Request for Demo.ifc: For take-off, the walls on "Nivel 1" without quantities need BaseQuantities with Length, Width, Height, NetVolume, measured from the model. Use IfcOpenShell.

First a look at what the model holds.

```python
import ifcopenshell
import ifcopenshell.util.element
import ifcopenshell.util.unit

model = ifcopenshell.open("Demo.ifc")
print(model.schema)
for unit_type in ("LENGTHUNIT", "AREAUNIT", "VOLUMEUNIT"):
    print(unit_type, ifcopenshell.util.unit.calculate_unit_scale(model, unit_type))
storey = next(s for s in model.by_type("IfcBuildingStorey") if s.Name == "Nivel 1")
walls = [e for e in ifcopenshell.util.element.get_decomposition(storey) if e.is_a("IfcWall")]
for e in sorted(walls, key=lambda e: e.id()):
    print(e.id(), e.is_a(), e.Name, list(ifcopenshell.util.element.get_psets(e, qtos_only=True)), sep=" | ")
```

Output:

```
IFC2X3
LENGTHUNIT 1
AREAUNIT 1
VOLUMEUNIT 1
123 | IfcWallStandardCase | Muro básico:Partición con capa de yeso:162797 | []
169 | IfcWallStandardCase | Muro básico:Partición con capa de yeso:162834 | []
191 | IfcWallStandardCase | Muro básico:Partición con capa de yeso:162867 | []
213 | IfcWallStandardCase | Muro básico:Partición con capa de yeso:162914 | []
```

```python
import ifcopenshell
import ifcopenshell.api.pset
import ifcopenshell.geom
import ifcopenshell.util.element
import ifcopenshell.util.shape
import ifcopenshell.util.unit

model = ifcopenshell.open("Demo.ifc")
unit_scale = ifcopenshell.util.unit.calculate_unit_scale(model)
volume_scale = ifcopenshell.util.unit.calculate_unit_scale(model, "VOLUMEUNIT")
settings = ifcopenshell.geom.settings()

storey = next(s for s in model.by_type("IfcBuildingStorey") if s.Name == "Nivel 1")
walls = [e for e in ifcopenshell.util.element.get_decomposition(storey) if e.is_a("IfcWall")]

for e in sorted(walls, key=lambda e: e.id()):
    if ifcopenshell.util.element.get_psets(e, qtos_only=True, should_inherit=False):
        continue
    # Geometry comes back in metres, in the element's own axes.
    shape = ifcopenshell.geom.create_shape(settings, e)
    values = {
        "Length": ifcopenshell.util.shape.get_x(shape.geometry) / unit_scale,
        "Width": ifcopenshell.util.shape.get_y(shape.geometry) / unit_scale,
        "Height": ifcopenshell.util.shape.get_z(shape.geometry) / unit_scale,
        "NetVolume": ifcopenshell.util.shape.get_volume(shape.geometry) / volume_scale,
    }
    qto = ifcopenshell.api.pset.add_qto(model, product=e, name="BaseQuantities")
    ifcopenshell.api.pset.edit_qto(model, qto=qto, properties=values)
    print(e.id(), {k: round(v, 3) for k, v in values.items()})

model.write("Demo_edited.ifc")
```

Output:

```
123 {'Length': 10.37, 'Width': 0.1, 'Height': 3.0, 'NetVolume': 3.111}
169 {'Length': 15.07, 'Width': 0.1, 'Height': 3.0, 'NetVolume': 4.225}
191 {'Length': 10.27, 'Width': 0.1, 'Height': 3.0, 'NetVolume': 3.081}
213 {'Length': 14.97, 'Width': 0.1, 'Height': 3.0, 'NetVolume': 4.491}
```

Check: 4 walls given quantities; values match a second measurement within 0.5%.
